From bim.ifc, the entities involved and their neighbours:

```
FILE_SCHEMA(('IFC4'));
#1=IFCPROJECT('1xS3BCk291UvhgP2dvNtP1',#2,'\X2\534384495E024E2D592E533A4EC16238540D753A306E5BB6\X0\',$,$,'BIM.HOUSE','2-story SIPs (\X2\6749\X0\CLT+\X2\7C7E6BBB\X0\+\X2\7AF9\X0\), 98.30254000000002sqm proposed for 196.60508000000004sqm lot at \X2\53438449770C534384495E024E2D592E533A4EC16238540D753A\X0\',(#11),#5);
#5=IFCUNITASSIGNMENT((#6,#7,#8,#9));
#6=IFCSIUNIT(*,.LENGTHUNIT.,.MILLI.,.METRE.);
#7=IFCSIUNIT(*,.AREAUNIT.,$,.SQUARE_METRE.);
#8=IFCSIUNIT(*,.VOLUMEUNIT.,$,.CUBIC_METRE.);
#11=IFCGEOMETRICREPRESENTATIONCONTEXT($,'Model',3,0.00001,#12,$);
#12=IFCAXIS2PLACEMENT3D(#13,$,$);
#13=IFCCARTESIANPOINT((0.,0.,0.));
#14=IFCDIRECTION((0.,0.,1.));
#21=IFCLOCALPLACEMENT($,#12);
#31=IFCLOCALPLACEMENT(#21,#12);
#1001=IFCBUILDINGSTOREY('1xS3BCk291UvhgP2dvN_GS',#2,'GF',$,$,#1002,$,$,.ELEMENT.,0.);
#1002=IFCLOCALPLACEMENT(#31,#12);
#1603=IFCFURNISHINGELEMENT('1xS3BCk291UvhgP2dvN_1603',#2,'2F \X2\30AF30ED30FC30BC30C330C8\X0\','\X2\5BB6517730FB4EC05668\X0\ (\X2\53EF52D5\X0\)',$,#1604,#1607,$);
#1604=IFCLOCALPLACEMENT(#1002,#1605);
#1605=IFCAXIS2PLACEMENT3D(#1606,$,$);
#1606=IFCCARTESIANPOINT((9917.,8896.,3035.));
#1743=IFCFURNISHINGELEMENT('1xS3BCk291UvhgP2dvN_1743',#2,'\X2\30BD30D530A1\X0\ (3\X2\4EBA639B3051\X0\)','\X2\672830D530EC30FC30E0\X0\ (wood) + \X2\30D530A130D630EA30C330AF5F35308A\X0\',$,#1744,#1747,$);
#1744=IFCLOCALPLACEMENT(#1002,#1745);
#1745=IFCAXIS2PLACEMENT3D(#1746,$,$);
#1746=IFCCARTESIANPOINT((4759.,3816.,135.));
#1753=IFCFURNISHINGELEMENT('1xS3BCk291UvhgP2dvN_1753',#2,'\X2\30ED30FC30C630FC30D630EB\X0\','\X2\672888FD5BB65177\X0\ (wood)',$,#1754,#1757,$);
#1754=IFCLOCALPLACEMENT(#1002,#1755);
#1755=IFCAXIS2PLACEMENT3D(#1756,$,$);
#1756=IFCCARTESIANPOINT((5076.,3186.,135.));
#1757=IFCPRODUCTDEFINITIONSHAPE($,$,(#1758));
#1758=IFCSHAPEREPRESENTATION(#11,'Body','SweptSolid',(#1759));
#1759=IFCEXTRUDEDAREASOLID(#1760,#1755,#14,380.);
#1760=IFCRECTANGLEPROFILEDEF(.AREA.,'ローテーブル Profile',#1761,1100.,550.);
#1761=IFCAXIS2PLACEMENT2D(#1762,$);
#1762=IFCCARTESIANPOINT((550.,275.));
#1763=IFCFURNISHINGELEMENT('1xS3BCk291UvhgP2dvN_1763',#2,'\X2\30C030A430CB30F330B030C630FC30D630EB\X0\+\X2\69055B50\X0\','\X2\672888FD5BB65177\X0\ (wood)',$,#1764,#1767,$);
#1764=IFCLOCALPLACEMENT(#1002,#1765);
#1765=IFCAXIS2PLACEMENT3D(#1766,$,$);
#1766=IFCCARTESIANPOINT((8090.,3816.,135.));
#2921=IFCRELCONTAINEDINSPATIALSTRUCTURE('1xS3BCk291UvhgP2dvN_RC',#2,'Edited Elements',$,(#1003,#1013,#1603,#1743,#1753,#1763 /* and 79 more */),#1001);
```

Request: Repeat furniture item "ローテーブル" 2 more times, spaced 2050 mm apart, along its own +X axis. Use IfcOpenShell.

```python
import ifcopenshell
import ifcopenshell.api.geometry
import ifcopenshell.api.root
import ifcopenshell.util.element
import ifcopenshell.util.placement
import ifcopenshell.util.unit

model = ifcopenshell.open("bim.ifc")
unit_scale = ifcopenshell.util.unit.calculate_unit_scale(model)


def reuse_history(source, copy):
    """copy_class also copies each property set's owner history, people and application; keep the originals."""
    for rel in copy.IsDefinedBy:
        if rel.is_a("IfcRelDefinesByProperties") and (history := rel.RelatingPropertyDefinition.OwnerHistory):
            rel.RelatingPropertyDefinition.OwnerHistory = source.OwnerHistory
            ifcopenshell.util.element.remove_deep2(model, history)


source = model.by_id(1753)
base = ifcopenshell.util.placement.get_local_placement(source.ObjectPlacement)
step = base[:3, 0] * 2.05 / unit_scale

for i in range(1, 3):
    copy = ifcopenshell.api.root.copy_class(model, product=source)
    copy.Representation = ifcopenshell.util.element.copy_deep(
        model, source.Representation, exclude=["IfcGeometricRepresentationContext", "IfcRepresentationMap"]
    )
    reuse_history(source, copy)
    matrix = base.copy()
    matrix[:3, 3] += i * step
    print("added at", matrix[:3, 3].round(3) + 0.0)
    ifcopenshell.api.geometry.edit_object_placement(model, product=copy, matrix=matrix, is_si=False)

model.write("bim_updated.ifc")
```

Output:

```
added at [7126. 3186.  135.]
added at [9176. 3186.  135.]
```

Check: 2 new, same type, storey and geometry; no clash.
